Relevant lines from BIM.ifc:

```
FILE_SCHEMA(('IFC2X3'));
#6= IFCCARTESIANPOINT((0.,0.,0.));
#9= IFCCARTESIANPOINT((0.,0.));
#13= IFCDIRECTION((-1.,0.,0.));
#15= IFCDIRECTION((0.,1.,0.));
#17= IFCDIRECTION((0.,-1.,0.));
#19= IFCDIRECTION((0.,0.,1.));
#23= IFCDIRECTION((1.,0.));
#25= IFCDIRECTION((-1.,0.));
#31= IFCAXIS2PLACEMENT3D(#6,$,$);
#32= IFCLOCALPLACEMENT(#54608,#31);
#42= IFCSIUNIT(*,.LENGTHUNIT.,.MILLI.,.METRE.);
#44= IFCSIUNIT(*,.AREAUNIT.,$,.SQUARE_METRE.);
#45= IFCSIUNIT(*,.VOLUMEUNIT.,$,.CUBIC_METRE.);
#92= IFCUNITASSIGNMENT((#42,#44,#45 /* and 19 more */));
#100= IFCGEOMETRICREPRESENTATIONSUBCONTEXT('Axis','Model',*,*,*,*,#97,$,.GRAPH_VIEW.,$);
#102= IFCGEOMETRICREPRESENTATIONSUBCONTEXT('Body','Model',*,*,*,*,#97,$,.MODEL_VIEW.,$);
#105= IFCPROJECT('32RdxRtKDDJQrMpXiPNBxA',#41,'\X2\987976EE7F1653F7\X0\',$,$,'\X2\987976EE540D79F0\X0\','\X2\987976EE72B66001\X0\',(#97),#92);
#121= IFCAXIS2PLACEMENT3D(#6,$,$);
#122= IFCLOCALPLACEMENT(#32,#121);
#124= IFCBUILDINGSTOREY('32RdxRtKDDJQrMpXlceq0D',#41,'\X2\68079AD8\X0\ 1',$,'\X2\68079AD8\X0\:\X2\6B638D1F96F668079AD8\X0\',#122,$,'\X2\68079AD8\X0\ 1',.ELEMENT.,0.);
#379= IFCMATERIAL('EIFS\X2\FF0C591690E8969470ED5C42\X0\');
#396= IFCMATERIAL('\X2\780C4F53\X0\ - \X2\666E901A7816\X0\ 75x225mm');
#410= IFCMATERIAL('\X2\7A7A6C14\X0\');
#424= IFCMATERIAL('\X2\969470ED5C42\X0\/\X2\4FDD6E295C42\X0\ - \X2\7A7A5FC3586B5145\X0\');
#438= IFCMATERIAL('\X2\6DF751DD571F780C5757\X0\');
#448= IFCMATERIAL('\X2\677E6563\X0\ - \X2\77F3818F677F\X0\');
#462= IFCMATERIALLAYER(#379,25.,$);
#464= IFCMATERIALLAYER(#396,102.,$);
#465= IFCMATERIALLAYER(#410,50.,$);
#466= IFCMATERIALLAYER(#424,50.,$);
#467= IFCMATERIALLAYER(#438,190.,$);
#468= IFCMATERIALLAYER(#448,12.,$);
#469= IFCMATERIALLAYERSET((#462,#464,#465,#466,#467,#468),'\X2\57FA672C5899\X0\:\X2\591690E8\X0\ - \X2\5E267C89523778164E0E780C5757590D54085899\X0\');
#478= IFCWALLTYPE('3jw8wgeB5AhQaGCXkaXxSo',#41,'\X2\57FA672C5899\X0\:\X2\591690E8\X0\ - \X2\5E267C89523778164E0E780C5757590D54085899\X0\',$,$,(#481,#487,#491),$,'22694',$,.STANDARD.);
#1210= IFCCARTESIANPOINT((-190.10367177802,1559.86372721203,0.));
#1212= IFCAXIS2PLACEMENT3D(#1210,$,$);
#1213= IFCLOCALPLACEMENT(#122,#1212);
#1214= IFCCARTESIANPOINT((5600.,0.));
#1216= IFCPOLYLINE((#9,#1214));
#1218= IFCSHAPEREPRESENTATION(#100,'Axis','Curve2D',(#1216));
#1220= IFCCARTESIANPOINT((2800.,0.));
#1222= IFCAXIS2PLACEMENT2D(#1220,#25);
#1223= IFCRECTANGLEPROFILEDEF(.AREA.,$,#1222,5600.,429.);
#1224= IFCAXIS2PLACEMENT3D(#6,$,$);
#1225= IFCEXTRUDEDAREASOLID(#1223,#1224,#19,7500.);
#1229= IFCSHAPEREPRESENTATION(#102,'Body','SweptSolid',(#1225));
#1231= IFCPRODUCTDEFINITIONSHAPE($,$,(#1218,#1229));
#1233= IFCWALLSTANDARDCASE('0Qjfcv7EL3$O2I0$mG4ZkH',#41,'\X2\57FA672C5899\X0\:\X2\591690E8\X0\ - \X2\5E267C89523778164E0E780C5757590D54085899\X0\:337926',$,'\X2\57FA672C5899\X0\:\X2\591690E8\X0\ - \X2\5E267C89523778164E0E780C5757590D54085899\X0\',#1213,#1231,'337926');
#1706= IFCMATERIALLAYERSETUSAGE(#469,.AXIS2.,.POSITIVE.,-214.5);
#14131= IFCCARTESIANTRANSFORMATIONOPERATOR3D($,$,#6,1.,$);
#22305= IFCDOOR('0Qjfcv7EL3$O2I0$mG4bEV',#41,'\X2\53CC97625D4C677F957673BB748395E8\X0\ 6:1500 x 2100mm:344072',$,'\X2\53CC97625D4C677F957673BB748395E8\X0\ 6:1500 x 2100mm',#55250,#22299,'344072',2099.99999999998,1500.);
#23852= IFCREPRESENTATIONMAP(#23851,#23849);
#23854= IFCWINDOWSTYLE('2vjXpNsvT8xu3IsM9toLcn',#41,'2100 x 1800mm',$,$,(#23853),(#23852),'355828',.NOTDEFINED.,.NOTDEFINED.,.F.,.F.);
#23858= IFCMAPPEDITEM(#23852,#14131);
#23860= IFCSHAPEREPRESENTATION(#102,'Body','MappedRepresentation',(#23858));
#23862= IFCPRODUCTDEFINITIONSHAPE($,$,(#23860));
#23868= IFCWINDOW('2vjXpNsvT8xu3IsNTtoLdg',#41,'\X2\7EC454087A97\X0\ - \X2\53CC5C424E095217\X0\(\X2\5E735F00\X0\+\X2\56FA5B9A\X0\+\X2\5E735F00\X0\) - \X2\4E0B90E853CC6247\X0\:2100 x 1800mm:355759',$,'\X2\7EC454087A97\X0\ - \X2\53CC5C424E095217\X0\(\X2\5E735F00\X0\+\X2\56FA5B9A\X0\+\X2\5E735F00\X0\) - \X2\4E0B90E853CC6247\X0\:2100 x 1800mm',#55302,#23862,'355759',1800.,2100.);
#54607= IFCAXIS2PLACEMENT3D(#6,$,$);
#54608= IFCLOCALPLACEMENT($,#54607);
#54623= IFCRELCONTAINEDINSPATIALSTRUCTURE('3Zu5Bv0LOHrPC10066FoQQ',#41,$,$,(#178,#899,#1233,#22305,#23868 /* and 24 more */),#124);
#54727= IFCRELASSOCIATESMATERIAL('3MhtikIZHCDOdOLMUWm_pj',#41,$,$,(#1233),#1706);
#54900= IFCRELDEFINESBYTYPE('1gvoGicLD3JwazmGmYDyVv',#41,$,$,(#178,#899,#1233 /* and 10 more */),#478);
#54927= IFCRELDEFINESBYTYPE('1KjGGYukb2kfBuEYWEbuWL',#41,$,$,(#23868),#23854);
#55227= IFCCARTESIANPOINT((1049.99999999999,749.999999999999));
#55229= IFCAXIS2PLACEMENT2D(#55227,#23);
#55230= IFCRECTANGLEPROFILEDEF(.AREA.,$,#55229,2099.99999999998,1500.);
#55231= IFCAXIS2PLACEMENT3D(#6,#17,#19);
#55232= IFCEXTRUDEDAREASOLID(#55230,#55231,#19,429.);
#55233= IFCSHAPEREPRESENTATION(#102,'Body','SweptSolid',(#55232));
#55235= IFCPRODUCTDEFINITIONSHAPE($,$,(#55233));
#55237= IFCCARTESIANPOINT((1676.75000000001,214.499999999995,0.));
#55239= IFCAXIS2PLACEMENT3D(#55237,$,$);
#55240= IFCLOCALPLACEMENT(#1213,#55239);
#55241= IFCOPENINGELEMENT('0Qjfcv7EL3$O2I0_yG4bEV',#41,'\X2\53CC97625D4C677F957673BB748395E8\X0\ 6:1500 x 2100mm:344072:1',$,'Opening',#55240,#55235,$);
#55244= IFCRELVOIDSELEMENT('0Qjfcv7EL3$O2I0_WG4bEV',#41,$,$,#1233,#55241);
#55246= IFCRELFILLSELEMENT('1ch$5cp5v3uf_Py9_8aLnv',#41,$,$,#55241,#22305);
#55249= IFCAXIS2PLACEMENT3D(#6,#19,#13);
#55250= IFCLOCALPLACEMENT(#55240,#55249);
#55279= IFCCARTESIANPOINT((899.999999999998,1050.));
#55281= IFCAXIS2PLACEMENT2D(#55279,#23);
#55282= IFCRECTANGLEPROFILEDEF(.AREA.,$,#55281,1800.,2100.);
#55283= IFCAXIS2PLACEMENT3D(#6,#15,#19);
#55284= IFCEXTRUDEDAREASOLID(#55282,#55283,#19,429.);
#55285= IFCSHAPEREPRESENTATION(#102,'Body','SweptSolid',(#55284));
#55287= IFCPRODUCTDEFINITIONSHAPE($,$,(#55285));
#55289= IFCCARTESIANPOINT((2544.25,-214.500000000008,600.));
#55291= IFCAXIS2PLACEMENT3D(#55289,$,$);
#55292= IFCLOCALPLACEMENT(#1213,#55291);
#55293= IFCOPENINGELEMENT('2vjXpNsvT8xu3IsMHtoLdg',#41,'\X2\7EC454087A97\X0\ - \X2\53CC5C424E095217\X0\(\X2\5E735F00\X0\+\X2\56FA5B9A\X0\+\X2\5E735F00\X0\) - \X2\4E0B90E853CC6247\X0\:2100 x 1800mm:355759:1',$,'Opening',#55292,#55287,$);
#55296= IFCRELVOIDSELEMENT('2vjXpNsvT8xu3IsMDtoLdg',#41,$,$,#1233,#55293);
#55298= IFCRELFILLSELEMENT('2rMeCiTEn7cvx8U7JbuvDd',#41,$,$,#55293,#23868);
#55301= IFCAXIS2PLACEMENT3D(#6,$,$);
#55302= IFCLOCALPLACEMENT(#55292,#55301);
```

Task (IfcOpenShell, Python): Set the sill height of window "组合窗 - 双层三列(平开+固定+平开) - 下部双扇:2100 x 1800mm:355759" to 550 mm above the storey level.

```python
import numpy as np
import ifcopenshell
import ifcopenshell.api.geometry
import ifcopenshell.geom
import ifcopenshell.util.element
import ifcopenshell.util.placement
import ifcopenshell.util.shape
import ifcopenshell.util.unit

model = ifcopenshell.open("BIM.ifc")
unit_scale = ifcopenshell.util.unit.calculate_unit_scale(model)

window = model.by_guid("2vjXpNsvT8xu3IsNTtoLdg")
opening = window.FillsVoids[0].RelatingOpeningElement
storey = ifcopenshell.util.element.get_container(window, ifc_class="IfcBuildingStorey")
level = ifcopenshell.util.placement.get_local_placement(storey.ObjectPlacement)[2, 3]

# The opening's origin need not be at the sill, so measure its lowest point.
shape = ifcopenshell.geom.create_shape(ifcopenshell.geom.settings(), opening)
bottom = ifcopenshell.util.shape.get_shape_bottom_elevation(shape, shape.geometry) / unit_scale
dz = level + 0.55 / unit_scale - bottom

shift = np.array([0.0, 0.0, dz])
# The window is placed relative to its opening, so it follows when the opening moves.
matrix = ifcopenshell.util.placement.get_local_placement(opening.ObjectPlacement)
matrix[:3, 3] += shift
ifcopenshell.api.geometry.edit_object_placement(
    model, product=opening, matrix=matrix, is_si=False, should_transform_children=True
)

print(f"moved by {dz * unit_scale:+.3f} m")

model.write("BIM_v2.ifc")
```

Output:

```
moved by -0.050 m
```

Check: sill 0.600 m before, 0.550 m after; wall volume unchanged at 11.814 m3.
